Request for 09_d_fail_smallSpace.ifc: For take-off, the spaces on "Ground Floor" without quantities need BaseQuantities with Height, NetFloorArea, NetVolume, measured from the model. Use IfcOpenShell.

First a look at what the model holds.

```python
import ifcopenshell
import ifcopenshell.util.element
import ifcopenshell.util.unit

model = ifcopenshell.open("09_d_fail_smallSpace.ifc")
print(model.schema)
for unit_type in ("LENGTHUNIT", "AREAUNIT", "VOLUMEUNIT"):
    print(unit_type, ifcopenshell.util.unit.calculate_unit_scale(model, unit_type))
storey = next(s for s in model.by_type("IfcBuildingStorey") if s.Name == "Ground Floor")
spaces = [e for e in ifcopenshell.util.element.get_decomposition(storey) if e.is_a("IfcSpace")]
for e in sorted(spaces, key=lambda e: e.id()):
    print(e.id(), e.is_a(), e.Name, list(ifcopenshell.util.element.get_psets(e, qtos_only=True)), sep=" | ")
```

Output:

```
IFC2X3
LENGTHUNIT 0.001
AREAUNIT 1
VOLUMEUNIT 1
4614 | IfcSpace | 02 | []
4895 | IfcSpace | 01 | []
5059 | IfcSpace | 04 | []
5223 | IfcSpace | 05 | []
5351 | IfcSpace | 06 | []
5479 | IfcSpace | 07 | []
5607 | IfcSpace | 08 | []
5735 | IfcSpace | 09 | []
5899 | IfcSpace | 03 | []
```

```python
import ifcopenshell
import ifcopenshell.api.pset
import ifcopenshell.geom
import ifcopenshell.util.element
import ifcopenshell.util.shape
import ifcopenshell.util.unit

model = ifcopenshell.open("09_d_fail_smallSpace.ifc")
unit_scale = ifcopenshell.util.unit.calculate_unit_scale(model)
area_scale = ifcopenshell.util.unit.calculate_unit_scale(model, "AREAUNIT")
volume_scale = ifcopenshell.util.unit.calculate_unit_scale(model, "VOLUMEUNIT")
settings = ifcopenshell.geom.settings()

storey = next(s for s in model.by_type("IfcBuildingStorey") if s.Name == "Ground Floor")
spaces = [e for e in ifcopenshell.util.element.get_decomposition(storey) if e.is_a("IfcSpace")]

for e in sorted(spaces, key=lambda e: e.id()):
    if ifcopenshell.util.element.get_psets(e, qtos_only=True, should_inherit=False):
        continue
    # Geometry comes back in metres, in the element's own axes.
    shape = ifcopenshell.geom.create_shape(settings, e)
    values = {
        "Height": ifcopenshell.util.shape.get_z(shape.geometry) / unit_scale,
        "NetFloorArea": ifcopenshell.util.shape.get_footprint_area(shape.geometry) / area_scale,
        "NetVolume": ifcopenshell.util.shape.get_volume(shape.geometry) / volume_scale,
    }
    qto = ifcopenshell.api.pset.add_qto(model, product=e, name="BaseQuantities")
    ifcopenshell.api.pset.edit_qto(model, qto=qto, properties=values)
    print(e.id(), {k: round(v, 3) for k, v in values.items()})

model.write("09_d_fail_smallSpace_updated.ifc")
```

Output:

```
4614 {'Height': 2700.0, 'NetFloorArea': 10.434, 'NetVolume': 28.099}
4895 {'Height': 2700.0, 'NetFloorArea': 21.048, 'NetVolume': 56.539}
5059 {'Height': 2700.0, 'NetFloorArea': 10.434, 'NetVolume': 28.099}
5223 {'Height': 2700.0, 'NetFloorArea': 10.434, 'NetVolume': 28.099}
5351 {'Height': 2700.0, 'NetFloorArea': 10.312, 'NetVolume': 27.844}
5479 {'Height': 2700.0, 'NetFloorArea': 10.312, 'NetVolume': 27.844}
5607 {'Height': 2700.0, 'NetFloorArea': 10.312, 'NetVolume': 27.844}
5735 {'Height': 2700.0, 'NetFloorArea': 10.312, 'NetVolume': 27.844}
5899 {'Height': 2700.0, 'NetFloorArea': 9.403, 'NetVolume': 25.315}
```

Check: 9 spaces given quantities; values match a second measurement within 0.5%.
